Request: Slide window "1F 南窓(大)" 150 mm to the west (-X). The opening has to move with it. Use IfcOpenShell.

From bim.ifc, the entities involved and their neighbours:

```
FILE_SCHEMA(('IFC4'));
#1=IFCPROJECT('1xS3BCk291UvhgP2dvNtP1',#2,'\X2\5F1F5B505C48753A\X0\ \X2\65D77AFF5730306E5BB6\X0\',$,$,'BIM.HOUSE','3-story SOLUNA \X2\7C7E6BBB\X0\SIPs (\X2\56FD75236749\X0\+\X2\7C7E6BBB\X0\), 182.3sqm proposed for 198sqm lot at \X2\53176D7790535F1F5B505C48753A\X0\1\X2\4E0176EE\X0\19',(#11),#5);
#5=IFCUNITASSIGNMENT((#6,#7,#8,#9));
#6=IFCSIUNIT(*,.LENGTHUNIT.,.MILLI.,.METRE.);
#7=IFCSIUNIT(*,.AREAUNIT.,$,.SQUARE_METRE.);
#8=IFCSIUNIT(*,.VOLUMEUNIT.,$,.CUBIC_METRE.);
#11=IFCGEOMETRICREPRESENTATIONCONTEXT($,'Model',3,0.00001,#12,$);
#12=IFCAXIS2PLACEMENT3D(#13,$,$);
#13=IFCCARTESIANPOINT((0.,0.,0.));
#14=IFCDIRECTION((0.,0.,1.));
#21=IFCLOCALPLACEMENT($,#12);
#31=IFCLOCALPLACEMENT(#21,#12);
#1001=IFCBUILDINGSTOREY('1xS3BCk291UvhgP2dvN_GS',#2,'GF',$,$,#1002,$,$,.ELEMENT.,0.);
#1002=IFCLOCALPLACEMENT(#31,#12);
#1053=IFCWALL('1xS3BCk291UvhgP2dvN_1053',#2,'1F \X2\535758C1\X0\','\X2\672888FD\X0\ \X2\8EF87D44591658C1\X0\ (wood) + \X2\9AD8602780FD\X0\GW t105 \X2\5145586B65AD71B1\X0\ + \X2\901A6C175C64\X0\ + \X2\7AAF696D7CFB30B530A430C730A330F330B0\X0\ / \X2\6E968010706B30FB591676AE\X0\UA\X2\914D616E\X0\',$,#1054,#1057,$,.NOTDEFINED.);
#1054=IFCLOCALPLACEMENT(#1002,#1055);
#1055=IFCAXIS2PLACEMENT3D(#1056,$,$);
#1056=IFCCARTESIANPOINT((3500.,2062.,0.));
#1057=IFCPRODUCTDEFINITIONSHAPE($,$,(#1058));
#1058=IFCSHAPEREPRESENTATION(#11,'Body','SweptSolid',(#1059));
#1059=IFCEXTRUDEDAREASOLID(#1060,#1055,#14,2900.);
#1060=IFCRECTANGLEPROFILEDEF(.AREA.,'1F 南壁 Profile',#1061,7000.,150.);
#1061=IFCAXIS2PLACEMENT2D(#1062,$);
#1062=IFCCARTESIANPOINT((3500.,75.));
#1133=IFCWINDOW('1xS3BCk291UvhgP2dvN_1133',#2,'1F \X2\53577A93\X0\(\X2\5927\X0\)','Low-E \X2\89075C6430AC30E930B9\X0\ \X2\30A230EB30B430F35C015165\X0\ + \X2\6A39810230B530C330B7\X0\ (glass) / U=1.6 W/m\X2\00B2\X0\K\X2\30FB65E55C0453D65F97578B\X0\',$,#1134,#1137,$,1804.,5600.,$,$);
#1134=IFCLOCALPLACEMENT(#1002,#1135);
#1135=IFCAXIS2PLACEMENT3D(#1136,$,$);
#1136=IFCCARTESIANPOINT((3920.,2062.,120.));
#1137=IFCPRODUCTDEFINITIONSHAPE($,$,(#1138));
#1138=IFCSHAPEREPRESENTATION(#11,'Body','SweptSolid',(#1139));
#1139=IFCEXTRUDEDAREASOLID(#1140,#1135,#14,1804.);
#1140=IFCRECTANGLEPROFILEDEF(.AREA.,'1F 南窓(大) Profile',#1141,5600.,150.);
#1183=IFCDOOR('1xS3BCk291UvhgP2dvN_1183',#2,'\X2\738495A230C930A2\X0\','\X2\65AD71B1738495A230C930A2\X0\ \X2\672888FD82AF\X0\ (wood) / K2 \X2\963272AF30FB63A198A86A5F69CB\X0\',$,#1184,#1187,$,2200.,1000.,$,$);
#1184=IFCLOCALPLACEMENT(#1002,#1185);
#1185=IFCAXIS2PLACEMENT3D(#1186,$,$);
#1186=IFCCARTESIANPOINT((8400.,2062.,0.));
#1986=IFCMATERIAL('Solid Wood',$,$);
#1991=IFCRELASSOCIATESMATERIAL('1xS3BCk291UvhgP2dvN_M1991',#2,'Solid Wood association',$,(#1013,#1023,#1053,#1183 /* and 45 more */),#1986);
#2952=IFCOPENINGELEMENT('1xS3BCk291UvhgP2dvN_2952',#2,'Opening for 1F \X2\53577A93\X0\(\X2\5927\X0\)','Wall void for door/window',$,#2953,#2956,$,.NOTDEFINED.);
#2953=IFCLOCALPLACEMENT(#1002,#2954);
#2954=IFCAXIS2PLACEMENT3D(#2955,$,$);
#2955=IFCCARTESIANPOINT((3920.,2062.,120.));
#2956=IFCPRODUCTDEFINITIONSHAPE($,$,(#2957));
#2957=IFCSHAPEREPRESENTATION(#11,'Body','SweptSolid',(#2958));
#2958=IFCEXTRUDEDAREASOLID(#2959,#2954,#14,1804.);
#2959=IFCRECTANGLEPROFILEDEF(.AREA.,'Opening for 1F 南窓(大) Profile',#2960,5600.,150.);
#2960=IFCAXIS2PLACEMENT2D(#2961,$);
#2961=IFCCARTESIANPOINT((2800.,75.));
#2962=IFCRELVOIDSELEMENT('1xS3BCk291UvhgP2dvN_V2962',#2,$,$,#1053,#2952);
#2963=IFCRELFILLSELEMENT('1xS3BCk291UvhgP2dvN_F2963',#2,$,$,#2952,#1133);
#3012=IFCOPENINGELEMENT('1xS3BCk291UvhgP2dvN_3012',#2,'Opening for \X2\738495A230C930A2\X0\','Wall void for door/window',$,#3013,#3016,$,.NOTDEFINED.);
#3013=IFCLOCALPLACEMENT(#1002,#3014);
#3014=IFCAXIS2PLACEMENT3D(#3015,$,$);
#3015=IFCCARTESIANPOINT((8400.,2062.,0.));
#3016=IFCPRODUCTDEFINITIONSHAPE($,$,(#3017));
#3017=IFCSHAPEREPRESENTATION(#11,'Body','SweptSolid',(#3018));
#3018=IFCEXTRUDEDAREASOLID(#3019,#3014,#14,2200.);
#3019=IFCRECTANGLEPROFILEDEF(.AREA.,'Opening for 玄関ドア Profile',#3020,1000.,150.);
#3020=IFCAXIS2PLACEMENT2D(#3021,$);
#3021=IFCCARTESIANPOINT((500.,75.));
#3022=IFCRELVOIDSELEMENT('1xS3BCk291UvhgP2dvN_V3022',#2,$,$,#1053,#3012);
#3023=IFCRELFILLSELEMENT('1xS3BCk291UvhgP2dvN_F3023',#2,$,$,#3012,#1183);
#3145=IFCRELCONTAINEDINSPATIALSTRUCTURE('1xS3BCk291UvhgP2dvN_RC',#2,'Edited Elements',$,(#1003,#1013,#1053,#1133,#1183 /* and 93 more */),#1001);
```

```python
import ifcopenshell
import ifcopenshell.api.geometry
import ifcopenshell.util.placement
import ifcopenshell.util.unit

model = ifcopenshell.open("bim.ifc")
unit_scale = ifcopenshell.util.unit.calculate_unit_scale(model)

window = model.by_id(1133)
opening = window.FillsVoids[0].RelatingOpeningElement
wall = opening.VoidsElements[0].RelatingBuildingElement

wall_matrix = ifcopenshell.util.placement.get_local_placement(wall.ObjectPlacement)
shift = wall_matrix[:3, 0] * -0.15 / unit_scale
before = ifcopenshell.util.placement.get_local_placement(window.ObjectPlacement)[:3, 3].copy()

# The window is not placed relative to its opening, so move both.
for product in (opening, window):
    matrix = ifcopenshell.util.placement.get_local_placement(product.ObjectPlacement)
    matrix[:3, 3] += shift
    ifcopenshell.api.geometry.edit_object_placement(model, product=product, matrix=matrix, is_si=False)

after = ifcopenshell.util.placement.get_local_placement(window.ObjectPlacement)[:3, 3]
print("window moved by", (after - before).round(3) + 0.0)

model.write("bim-out.ifc")
```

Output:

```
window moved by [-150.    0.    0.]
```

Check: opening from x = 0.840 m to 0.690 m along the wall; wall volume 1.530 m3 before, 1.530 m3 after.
